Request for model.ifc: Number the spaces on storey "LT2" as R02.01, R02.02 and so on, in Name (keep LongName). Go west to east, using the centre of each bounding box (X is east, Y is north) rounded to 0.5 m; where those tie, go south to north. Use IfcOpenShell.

First a look at what the model holds.

```python
import ifcopenshell
import ifcopenshell.util.element
import ifcopenshell.util.placement

model = ifcopenshell.open("model.ifc")
print(model.schema)
storey = next(s for s in model.by_type("IfcBuildingStorey") if s.Name == "LT2")
spaces = [e for e in ifcopenshell.util.element.get_decomposition(storey) if e.is_a("IfcSpace")]
for e in sorted(spaces, key=lambda e: e.id()):
    origin = ifcopenshell.util.placement.get_local_placement(e.ObjectPlacement)[:3, 3]
    print(e.id(), e.Name, e.LongName, origin.round(2) + 0.0, sep=" | ")
```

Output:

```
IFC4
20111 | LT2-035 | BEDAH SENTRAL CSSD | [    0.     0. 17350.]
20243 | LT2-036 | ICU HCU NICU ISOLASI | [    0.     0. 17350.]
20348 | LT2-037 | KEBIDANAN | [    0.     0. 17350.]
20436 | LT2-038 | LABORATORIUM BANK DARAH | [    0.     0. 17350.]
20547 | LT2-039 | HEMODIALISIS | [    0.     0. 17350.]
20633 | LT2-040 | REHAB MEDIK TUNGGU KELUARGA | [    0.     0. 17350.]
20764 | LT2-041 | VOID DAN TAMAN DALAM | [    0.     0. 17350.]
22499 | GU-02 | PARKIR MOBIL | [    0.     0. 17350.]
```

```python
import ifcopenshell
import ifcopenshell.geom
import ifcopenshell.util.element
import ifcopenshell.util.shape

model = ifcopenshell.open("model.ifc")
settings = ifcopenshell.geom.settings()
settings.set("use-world-coords", True)


def centre(element):
    shape = ifcopenshell.geom.create_shape(settings, element)
    return ifcopenshell.util.shape.get_bbox_centroid(shape.geometry)


storey = next(s for s in model.by_type("IfcBuildingStorey") if s.Name == "LT2")
spaces = [e for e in ifcopenshell.util.element.get_decomposition(storey) if e.is_a("IfcSpace")]

# Insertion points can sit at a corner or the storey origin, so sort by the geometry (in metres).
centres = {e: centre(e) for e in spaces}
spaces.sort(key=lambda e: (round(centres[e][0] / 0.5), centres[e][1]))

for i, e in enumerate(spaces, start=1):
    number = f"R02.{i:02d}"
    e.Name = number
    print(e.id(), number)

model.write("model-out.ifc")
```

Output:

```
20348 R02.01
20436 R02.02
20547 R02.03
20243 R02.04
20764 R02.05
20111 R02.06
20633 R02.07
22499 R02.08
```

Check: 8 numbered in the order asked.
